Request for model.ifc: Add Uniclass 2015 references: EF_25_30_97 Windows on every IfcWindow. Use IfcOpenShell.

First a look at what the model holds.

```python
import ifcopenshell

model = ifcopenshell.open("model.ifc")
print(model.schema)
print("classifications:", [c.Name for c in model.by_type("IfcClassification")])
for ifc_class in ("IfcDoor", "IfcRoof", "IfcStair", "IfcWall", "IfcWindow"):
    print(ifc_class, len(model.by_type(ifc_class)))
```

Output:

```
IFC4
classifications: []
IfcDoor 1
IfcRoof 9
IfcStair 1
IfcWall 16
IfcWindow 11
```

```python
import ifcopenshell
import ifcopenshell.api.classification

model = ifcopenshell.open("model.ifc")

system = ifcopenshell.api.classification.add_classification(model, classification="Uniclass 2015")

codes = {
    "IfcWindow": ("EF_25_30_97", "Windows"),
}
for ifc_class, (code, name) in codes.items():
    products = model.by_type(ifc_class)
    ifcopenshell.api.classification.add_reference(
        model, products=products, classification=system, identification=code, name=name
    )
    print(code, len(products))

model.write("model_v2.ifc")
```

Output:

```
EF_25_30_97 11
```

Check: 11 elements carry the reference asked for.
